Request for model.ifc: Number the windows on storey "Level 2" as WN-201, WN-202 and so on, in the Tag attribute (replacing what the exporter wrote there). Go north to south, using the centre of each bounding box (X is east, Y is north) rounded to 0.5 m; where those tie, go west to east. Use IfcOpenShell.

First a look at what the model holds.

```python
import ifcopenshell
import ifcopenshell.util.element
import ifcopenshell.util.placement

model = ifcopenshell.open("model.ifc")
print(model.schema)
storey = next(s for s in model.by_type("IfcBuildingStorey") if s.Name == "Level 2")
windows = [e for e in ifcopenshell.util.element.get_decomposition(storey) if e.is_a("IfcWindow")]
for e in sorted(windows, key=lambda e: e.id()):
    origin = ifcopenshell.util.placement.get_local_placement(e.ObjectPlacement)[:3, 3]
    print(e.id(), e.Tag, e.Name, origin.round(2) + 0.0, sep=" | ")
```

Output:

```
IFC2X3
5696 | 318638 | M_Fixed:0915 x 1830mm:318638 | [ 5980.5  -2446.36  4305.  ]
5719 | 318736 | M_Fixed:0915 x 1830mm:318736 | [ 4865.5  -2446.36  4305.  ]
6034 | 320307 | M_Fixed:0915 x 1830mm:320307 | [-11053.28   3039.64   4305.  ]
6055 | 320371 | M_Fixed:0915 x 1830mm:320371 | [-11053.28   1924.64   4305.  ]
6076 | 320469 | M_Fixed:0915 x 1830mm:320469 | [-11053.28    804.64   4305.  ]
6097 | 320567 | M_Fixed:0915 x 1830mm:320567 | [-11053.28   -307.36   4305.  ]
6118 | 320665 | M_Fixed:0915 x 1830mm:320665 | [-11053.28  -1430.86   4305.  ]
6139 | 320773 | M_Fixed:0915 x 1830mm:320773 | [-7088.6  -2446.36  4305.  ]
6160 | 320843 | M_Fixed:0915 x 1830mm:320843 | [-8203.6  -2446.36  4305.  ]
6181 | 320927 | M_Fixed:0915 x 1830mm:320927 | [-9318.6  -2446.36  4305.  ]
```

```python
import ifcopenshell
import ifcopenshell.geom
import ifcopenshell.util.element
import ifcopenshell.util.shape

model = ifcopenshell.open("model.ifc")
settings = ifcopenshell.geom.settings()
settings.set("use-world-coords", True)


def centre(element):
    shape = ifcopenshell.geom.create_shape(settings, element)
    return ifcopenshell.util.shape.get_bbox_centroid(shape.geometry)


storey = next(s for s in model.by_type("IfcBuildingStorey") if s.Name == "Level 2")
windows = [e for e in ifcopenshell.util.element.get_decomposition(storey) if e.is_a("IfcWindow")]

# Insertion points can sit at a corner or the storey origin, so sort by the geometry (in metres).
centres = {e: centre(e) for e in windows}
windows.sort(key=lambda e: (-round(centres[e][1] / 0.5), centres[e][0]))

for i, e in enumerate(windows, start=1):
    number = f"WN-2{i:02d}"
    e.Tag = number
    print(e.id(), number)

model.write("model_updated.ifc")
```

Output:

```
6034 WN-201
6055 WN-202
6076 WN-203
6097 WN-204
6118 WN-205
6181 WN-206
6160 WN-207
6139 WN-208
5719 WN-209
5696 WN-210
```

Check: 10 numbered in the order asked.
